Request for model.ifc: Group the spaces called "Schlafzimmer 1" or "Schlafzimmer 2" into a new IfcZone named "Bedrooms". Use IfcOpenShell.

First a look at what the model holds.

```python
import ifcopenshell

model = ifcopenshell.open("model.ifc")
print(model.schema)
seen = {}
for space in model.by_type("IfcSpace"):
    seen[space.LongName] = seen.get(space.LongName, 0) + 1
for name, count in sorted(seen.items(), key=str):
    print(count, "x", name)
print("zones:", [z.Name for z in model.by_type("IfcZone")][:20])
```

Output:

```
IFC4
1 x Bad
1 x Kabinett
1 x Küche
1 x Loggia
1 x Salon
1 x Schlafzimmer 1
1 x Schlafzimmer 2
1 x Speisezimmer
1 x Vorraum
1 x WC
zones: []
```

```python
import ifcopenshell
import ifcopenshell.api.group
import ifcopenshell.api.root

model = ifcopenshell.open("model.ifc")

names = {"Schlafzimmer 1", "Schlafzimmer 2"}
spaces = [s for s in model.by_type("IfcSpace") if s.LongName in names]

zone = ifcopenshell.api.root.create_entity(model, ifc_class="IfcZone", name="Bedrooms")
ifcopenshell.api.group.assign_group(model, products=spaces, group=zone)
print(len(spaces), "spaces in", zone.Name)

model.write("model_rev.ifc")
```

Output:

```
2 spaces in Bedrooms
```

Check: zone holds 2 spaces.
